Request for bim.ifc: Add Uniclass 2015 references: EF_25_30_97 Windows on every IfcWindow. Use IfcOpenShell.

First a look at what the model holds.

```python
import ifcopenshell

model = ifcopenshell.open("bim.ifc")
print(model.schema)
print("classifications:", [c.Name for c in model.by_type("IfcClassification")])
for ifc_class in ("IfcDoor", "IfcRoof", "IfcStair", "IfcWall", "IfcWindow"):
    print(ifc_class, len(model.by_type(ifc_class)))
```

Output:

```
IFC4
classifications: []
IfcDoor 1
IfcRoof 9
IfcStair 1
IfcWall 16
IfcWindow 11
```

```python
import ifcopenshell
import ifcopenshell.api.classification

model = ifcopenshell.open("bim.ifc")

system = ifcopenshell.api.classification.add_classification(model, classification="Uniclass 2015")

codes = {
    "IfcWindow": ("EF_25_30_97", "Windows"),
}
for ifc_class, (code, name) in codes.items():
    products = model.by_type(ifc_class)
    ifcopenshell.api.classification.add_reference(
        model, products=products, classification=system, identification=code, name=name
    )
    print(code, len(products))

model.write("bim_updated.ifc")
```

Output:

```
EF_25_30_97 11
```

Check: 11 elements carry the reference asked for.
